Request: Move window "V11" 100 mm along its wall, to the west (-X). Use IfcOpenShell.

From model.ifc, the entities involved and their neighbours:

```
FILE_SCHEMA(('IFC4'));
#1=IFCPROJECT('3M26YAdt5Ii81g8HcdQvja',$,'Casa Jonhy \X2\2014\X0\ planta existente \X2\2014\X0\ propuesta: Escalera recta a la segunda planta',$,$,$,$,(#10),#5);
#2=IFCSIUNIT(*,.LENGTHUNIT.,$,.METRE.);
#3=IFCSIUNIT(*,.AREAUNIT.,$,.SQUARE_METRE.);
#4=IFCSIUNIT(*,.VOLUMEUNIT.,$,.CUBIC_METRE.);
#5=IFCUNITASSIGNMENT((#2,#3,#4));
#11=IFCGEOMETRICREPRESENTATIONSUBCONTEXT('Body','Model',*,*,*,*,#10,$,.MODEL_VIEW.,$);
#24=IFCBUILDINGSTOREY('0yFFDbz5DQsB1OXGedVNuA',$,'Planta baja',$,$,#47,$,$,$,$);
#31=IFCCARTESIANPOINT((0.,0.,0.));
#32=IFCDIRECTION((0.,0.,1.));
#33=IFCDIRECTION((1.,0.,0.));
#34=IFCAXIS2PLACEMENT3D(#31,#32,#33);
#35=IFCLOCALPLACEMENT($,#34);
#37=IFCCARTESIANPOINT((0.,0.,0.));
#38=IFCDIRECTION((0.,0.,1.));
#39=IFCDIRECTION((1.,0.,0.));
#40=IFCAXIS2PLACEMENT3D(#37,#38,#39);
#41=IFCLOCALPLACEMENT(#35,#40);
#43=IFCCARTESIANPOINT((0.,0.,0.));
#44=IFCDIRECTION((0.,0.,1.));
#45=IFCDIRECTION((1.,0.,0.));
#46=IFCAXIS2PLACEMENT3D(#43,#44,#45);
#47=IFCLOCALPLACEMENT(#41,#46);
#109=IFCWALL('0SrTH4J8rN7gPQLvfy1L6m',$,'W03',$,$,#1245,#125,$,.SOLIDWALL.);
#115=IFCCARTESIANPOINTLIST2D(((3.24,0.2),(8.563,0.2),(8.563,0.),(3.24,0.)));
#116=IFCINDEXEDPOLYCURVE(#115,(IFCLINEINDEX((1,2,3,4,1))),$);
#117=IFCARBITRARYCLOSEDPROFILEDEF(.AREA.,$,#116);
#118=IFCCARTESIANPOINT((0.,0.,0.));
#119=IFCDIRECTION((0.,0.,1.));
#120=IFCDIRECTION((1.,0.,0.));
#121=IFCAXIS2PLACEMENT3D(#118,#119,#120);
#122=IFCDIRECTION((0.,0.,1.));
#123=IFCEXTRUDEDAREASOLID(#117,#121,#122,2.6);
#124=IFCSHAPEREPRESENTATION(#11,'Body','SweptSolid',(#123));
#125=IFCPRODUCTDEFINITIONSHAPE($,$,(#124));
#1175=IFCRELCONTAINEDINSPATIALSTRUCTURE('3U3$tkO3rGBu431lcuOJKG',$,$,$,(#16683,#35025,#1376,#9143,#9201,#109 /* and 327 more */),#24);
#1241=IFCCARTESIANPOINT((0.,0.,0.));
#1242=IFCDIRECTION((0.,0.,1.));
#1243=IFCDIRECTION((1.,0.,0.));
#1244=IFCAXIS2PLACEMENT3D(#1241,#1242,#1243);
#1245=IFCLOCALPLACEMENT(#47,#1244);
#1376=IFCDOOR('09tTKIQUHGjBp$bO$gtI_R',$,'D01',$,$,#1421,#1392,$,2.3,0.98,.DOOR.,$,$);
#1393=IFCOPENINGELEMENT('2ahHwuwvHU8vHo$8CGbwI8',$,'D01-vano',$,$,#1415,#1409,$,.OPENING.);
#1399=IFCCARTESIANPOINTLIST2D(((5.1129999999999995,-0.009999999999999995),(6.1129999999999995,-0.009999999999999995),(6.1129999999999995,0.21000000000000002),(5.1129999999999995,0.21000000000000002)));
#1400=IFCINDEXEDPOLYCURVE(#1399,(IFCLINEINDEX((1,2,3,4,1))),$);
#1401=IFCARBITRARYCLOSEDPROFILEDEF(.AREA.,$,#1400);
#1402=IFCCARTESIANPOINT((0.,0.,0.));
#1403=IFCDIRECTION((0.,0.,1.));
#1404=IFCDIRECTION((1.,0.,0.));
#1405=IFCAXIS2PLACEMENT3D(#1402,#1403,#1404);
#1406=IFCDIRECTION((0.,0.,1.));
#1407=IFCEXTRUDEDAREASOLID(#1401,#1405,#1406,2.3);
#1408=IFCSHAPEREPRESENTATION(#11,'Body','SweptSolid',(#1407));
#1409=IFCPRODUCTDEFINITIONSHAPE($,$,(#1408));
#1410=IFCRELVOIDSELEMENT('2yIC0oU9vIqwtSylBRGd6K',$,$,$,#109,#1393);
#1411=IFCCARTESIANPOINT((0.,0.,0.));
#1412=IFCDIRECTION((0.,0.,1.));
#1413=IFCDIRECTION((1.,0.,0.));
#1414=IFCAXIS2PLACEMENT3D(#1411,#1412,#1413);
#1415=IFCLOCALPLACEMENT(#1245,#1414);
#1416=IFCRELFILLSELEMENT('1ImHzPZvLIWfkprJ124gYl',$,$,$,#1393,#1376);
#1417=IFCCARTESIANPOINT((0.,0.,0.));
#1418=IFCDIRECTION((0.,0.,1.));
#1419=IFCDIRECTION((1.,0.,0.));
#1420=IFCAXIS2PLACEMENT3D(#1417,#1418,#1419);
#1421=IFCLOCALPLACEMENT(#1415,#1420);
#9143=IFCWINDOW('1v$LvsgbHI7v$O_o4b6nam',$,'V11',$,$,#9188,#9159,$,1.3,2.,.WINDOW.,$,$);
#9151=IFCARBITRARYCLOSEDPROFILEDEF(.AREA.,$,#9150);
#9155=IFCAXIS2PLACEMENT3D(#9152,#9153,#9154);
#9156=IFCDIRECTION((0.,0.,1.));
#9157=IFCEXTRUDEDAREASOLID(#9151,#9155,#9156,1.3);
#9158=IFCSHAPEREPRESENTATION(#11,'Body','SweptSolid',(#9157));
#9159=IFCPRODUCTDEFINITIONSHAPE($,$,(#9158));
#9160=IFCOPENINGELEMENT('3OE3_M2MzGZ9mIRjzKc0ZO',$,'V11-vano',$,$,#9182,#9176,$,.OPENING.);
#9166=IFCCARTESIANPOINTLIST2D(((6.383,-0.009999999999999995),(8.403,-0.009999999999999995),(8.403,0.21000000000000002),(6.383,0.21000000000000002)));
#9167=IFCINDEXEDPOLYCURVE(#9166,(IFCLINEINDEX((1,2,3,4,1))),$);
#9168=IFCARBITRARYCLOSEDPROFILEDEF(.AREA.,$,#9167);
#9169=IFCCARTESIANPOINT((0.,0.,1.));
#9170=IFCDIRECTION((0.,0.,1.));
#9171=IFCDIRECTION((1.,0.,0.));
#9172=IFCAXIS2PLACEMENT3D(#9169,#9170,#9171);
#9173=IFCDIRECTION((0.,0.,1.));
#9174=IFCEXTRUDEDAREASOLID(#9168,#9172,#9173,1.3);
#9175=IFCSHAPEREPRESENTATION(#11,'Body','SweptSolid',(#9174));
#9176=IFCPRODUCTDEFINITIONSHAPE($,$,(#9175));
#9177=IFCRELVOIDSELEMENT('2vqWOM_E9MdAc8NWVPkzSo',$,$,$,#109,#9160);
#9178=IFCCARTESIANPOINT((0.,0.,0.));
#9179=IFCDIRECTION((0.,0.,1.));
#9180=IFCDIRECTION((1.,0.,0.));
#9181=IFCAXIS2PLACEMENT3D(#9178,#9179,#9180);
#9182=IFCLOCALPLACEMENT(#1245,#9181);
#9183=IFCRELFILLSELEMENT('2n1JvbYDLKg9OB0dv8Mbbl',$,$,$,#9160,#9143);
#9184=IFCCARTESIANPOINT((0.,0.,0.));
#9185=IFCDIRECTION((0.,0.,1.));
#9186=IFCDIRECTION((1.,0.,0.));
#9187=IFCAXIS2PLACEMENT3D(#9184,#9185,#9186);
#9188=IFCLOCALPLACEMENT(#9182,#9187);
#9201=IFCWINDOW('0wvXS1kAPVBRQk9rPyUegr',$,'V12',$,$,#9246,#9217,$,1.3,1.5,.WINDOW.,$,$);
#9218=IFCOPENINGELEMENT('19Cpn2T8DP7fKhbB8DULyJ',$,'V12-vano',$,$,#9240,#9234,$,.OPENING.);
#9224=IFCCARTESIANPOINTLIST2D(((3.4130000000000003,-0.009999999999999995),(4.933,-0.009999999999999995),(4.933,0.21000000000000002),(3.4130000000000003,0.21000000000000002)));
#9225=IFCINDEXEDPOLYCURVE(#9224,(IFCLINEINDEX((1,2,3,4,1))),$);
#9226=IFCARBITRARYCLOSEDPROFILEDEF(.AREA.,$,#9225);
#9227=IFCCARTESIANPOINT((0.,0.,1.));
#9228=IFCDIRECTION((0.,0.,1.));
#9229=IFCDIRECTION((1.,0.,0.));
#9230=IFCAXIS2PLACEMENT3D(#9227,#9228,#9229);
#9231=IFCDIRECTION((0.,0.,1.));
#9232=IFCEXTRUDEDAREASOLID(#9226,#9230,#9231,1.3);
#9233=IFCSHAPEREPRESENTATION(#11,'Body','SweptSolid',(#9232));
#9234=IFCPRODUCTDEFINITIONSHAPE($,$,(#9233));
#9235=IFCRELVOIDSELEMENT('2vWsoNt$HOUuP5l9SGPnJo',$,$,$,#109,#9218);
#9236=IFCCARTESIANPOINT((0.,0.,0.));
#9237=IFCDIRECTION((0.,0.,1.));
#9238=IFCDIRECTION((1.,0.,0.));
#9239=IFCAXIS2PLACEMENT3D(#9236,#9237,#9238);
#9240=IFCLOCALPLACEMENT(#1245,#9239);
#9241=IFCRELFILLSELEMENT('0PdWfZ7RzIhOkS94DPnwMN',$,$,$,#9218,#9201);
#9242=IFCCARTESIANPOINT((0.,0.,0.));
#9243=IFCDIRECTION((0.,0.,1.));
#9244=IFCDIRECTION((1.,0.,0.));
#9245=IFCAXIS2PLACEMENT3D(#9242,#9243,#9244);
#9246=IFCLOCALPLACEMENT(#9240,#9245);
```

```python
import ifcopenshell
import ifcopenshell.api.geometry
import ifcopenshell.util.placement
import ifcopenshell.util.unit

model = ifcopenshell.open("model.ifc")
unit_scale = ifcopenshell.util.unit.calculate_unit_scale(model)

window = model.by_id(9143)
opening = window.FillsVoids[0].RelatingOpeningElement
wall = opening.VoidsElements[0].RelatingBuildingElement

wall_matrix = ifcopenshell.util.placement.get_local_placement(wall.ObjectPlacement)
shift = wall_matrix[:3, 0] * -0.1 / unit_scale
before = ifcopenshell.util.placement.get_local_placement(window.ObjectPlacement)[:3, 3].copy()

# The window is placed relative to its opening, so it follows when the opening moves.
matrix = ifcopenshell.util.placement.get_local_placement(opening.ObjectPlacement)
matrix[:3, 3] += shift
ifcopenshell.api.geometry.edit_object_placement(
    model, product=opening, matrix=matrix, is_si=False, should_transform_children=True
)

after = ifcopenshell.util.placement.get_local_placement(window.ObjectPlacement)[:3, 3]
print("window moved by", (after - before).round(3) + 0.0)

model.write("model_updated.ifc")
```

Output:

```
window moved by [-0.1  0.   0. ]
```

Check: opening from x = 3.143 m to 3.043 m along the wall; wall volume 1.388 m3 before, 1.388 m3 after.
